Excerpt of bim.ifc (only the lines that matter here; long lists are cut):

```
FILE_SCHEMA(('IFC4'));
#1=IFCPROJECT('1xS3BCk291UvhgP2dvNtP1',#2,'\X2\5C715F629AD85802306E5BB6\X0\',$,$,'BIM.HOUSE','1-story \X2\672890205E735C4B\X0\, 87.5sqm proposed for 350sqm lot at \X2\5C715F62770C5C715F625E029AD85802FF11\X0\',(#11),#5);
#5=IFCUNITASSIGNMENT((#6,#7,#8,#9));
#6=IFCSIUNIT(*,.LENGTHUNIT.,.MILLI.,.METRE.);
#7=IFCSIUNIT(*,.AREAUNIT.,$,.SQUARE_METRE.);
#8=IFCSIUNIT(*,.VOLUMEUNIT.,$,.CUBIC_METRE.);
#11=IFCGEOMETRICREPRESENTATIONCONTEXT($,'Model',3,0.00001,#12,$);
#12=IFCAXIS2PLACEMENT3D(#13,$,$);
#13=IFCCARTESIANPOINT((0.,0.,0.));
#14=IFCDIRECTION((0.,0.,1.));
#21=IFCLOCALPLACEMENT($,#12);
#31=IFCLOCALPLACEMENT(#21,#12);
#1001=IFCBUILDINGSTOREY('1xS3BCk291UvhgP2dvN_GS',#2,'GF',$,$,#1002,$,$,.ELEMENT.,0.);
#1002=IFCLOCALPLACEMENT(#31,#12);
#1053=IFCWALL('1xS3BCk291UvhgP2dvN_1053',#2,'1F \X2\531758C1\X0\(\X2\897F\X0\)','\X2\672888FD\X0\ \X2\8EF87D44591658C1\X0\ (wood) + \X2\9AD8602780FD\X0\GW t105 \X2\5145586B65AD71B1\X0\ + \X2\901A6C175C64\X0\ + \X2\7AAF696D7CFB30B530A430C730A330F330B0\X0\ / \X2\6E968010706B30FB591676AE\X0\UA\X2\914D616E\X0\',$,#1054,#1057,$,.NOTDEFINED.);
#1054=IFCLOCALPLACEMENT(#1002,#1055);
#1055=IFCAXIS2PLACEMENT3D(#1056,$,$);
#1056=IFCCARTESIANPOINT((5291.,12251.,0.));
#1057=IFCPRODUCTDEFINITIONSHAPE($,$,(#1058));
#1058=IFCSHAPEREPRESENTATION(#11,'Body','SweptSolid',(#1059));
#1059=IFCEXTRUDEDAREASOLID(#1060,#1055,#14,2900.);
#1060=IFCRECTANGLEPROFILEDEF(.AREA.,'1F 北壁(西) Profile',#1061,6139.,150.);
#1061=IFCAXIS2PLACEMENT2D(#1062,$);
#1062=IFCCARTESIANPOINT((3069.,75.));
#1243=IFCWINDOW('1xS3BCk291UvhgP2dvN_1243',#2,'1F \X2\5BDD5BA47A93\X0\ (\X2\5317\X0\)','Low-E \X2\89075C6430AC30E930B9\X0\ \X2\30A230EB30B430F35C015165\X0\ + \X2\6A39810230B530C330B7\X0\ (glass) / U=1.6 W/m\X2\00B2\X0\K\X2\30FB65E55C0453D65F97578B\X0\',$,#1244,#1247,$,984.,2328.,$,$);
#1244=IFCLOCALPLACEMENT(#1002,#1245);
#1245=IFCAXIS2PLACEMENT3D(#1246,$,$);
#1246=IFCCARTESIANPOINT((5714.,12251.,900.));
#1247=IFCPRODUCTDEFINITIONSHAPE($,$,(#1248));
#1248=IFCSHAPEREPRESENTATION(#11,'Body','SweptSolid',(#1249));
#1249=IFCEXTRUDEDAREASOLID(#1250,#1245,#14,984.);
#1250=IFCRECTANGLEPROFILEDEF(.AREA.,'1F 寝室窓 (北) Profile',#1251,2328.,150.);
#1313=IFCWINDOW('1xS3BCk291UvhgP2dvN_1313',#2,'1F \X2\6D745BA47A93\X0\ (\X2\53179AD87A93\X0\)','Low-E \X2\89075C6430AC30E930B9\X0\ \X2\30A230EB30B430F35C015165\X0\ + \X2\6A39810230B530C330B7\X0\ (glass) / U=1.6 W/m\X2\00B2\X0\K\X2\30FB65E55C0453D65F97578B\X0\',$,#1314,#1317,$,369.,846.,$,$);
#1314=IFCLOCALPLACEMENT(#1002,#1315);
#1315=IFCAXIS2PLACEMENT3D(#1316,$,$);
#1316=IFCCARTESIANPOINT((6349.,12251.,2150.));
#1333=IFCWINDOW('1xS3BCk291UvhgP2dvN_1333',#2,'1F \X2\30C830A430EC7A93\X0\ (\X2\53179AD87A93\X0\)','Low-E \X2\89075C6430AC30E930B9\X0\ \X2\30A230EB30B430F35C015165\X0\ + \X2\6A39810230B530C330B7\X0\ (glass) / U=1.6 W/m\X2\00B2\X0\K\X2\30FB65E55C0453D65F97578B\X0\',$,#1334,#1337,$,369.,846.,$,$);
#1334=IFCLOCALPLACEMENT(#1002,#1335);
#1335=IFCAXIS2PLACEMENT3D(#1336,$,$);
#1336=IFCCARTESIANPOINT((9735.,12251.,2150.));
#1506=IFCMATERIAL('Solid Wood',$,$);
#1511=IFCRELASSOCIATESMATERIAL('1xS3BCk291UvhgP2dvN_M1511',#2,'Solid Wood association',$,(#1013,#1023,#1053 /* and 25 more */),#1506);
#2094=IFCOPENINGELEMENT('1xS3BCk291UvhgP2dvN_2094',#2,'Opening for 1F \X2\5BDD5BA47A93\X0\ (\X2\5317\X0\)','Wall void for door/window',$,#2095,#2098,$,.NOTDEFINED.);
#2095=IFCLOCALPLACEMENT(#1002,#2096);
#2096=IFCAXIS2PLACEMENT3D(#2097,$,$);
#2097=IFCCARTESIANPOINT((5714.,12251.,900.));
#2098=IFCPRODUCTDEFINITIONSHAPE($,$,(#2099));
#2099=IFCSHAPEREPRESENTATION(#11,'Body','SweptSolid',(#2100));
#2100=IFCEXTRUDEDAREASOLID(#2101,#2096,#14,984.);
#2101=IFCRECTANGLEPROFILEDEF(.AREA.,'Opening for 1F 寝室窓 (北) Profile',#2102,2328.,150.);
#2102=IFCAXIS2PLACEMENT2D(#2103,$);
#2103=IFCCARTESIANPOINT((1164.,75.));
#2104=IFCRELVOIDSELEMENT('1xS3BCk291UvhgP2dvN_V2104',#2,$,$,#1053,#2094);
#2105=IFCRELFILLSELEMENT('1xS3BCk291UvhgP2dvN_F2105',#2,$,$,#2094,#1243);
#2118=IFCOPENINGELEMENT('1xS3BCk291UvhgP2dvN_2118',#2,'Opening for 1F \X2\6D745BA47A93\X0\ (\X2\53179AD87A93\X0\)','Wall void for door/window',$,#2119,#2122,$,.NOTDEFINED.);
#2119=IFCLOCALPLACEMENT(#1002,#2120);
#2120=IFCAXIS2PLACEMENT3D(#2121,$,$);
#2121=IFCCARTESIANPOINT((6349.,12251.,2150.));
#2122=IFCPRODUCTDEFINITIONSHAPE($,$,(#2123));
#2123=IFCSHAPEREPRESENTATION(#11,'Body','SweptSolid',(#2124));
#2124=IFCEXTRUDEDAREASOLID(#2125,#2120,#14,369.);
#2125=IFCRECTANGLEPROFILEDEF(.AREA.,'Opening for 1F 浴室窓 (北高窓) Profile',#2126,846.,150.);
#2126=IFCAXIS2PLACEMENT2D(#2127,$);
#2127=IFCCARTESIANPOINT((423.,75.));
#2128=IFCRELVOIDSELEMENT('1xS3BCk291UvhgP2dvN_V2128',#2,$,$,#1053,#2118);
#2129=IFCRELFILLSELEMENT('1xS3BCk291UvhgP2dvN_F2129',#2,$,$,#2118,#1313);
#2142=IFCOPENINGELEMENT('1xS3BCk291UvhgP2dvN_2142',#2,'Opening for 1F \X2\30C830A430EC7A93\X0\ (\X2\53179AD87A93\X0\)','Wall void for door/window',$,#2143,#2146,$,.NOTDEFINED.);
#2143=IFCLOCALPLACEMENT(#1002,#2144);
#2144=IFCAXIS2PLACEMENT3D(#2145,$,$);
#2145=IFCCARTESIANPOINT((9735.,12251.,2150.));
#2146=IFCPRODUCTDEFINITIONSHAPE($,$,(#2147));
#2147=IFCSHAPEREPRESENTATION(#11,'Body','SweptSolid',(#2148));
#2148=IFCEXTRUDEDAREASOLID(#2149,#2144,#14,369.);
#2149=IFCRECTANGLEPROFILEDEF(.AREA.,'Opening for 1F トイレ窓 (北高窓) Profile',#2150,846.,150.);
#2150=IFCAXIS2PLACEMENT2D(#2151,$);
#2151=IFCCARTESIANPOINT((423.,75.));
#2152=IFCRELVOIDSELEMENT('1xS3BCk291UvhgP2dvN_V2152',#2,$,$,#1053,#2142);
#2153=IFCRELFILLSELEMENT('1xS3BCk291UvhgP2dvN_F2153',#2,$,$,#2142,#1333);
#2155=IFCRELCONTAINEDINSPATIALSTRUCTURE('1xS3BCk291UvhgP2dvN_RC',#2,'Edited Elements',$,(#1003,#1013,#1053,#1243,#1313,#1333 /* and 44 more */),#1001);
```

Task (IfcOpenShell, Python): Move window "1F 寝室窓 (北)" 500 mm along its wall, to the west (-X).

```python
import ifcopenshell
import ifcopenshell.api.geometry
import ifcopenshell.util.placement
import ifcopenshell.util.unit

model = ifcopenshell.open("bim.ifc")
unit_scale = ifcopenshell.util.unit.calculate_unit_scale(model)

window = model.by_guid("1xS3BCk291UvhgP2dvN_1243")
opening = window.FillsVoids[0].RelatingOpeningElement
wall = opening.VoidsElements[0].RelatingBuildingElement

wall_matrix = ifcopenshell.util.placement.get_local_placement(wall.ObjectPlacement)
shift = wall_matrix[:3, 0] * -0.5 / unit_scale
before = ifcopenshell.util.placement.get_local_placement(window.ObjectPlacement)[:3, 3].copy()

# The window is not placed relative to its opening, so move both.
for product in (opening, window):
    matrix = ifcopenshell.util.placement.get_local_placement(product.ObjectPlacement)
    matrix[:3, 3] += shift
    ifcopenshell.api.geometry.edit_object_placement(model, product=product, matrix=matrix, is_si=False)

after = ifcopenshell.util.placement.get_local_placement(window.ObjectPlacement)[:3, 3]
print("window moved by", (after - before).round(3) + 0.0)

model.write("bim_rev.ifc")
```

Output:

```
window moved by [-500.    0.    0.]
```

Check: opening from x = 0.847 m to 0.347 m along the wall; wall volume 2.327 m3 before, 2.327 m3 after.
